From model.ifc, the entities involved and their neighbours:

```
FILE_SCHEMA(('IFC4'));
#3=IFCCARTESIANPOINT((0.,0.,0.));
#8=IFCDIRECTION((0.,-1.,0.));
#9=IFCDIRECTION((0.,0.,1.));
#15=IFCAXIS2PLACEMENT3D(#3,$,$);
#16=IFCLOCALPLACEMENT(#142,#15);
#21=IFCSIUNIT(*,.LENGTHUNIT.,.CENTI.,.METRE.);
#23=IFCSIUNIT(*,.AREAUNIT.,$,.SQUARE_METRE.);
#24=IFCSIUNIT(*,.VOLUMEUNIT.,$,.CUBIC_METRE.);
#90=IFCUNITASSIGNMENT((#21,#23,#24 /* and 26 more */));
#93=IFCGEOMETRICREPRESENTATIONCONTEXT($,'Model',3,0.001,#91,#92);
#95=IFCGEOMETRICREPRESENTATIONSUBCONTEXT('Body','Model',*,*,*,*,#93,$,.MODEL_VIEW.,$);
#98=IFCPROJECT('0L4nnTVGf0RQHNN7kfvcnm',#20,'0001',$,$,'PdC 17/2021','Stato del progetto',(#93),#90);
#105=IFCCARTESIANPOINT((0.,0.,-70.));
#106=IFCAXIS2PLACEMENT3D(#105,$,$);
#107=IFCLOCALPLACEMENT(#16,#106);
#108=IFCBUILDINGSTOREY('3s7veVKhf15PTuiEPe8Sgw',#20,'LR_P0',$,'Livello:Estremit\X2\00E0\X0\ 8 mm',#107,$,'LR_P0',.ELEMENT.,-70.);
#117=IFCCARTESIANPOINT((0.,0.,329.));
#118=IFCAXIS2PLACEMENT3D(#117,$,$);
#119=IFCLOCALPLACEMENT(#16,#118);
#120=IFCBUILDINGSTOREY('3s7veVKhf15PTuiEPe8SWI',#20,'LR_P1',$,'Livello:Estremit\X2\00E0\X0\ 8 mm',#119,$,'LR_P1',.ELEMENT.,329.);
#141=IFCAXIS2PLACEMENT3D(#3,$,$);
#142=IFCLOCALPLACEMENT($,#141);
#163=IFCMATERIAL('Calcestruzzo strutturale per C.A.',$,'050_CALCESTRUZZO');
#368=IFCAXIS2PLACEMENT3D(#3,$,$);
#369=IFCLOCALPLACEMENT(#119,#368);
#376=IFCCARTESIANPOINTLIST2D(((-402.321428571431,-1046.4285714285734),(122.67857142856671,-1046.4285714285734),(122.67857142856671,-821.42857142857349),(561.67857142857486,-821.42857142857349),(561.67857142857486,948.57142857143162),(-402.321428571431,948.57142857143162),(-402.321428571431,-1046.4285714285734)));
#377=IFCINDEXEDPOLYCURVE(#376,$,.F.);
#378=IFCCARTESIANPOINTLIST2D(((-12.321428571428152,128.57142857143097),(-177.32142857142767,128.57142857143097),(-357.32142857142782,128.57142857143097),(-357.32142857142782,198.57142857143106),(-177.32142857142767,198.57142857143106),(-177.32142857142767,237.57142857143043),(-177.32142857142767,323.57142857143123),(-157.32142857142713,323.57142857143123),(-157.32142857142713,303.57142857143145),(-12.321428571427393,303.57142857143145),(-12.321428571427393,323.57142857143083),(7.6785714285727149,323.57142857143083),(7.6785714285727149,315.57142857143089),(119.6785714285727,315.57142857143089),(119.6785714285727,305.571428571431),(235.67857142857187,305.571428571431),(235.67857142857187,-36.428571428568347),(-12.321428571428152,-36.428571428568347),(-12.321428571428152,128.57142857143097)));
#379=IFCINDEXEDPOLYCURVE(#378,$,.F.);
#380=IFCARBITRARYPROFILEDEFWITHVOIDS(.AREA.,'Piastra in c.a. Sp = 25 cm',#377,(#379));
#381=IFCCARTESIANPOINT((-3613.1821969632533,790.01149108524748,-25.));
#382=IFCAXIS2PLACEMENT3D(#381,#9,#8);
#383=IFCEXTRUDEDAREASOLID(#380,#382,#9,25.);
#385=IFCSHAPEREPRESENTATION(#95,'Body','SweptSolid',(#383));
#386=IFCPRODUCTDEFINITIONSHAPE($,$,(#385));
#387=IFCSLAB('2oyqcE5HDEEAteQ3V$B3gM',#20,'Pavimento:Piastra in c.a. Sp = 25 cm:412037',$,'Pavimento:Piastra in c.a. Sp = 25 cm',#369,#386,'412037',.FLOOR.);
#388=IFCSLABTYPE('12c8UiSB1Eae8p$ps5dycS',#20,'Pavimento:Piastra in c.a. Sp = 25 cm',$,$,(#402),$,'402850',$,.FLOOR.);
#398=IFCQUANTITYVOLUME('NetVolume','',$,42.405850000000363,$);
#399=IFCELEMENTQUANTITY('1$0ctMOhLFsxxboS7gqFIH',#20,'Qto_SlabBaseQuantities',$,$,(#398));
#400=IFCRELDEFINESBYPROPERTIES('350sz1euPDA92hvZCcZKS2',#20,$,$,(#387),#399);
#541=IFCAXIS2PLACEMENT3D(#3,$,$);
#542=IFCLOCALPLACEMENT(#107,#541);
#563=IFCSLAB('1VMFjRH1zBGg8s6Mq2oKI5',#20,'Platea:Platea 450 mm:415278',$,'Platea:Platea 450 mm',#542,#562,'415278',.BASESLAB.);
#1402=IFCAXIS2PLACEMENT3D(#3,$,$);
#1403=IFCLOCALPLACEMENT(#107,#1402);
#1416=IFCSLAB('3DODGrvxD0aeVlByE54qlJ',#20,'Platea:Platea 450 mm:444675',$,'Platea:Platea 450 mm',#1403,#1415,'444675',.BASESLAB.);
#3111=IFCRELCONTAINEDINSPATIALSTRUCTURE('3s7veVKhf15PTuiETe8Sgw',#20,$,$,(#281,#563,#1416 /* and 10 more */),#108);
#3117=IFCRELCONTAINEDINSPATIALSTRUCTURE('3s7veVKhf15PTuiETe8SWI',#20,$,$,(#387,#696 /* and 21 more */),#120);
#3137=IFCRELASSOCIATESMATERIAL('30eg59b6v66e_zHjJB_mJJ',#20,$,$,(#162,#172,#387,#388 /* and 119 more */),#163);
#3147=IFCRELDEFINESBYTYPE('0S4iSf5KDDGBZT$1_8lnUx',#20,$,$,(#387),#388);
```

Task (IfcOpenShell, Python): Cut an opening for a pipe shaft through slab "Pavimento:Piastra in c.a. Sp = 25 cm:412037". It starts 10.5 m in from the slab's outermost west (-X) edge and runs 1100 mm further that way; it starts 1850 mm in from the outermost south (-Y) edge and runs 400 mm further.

```python
import numpy as np
import ifcopenshell
import ifcopenshell.api.feature
import ifcopenshell.api.geometry
import ifcopenshell.api.pset
import ifcopenshell.api.root
import ifcopenshell.geom
import ifcopenshell.util.element
import ifcopenshell.util.placement
import ifcopenshell.util.representation
import ifcopenshell.util.shape
import ifcopenshell.util.unit

model = ifcopenshell.open("model.ifc")
unit_scale = ifcopenshell.util.unit.calculate_unit_scale(model)
volume_scale = ifcopenshell.util.unit.calculate_unit_scale(model, "VOLUMEUNIT")
settings = ifcopenshell.geom.settings()


def volume(element):
    """Net volume in cubic metres, openings subtracted."""
    shape = ifcopenshell.geom.create_shape(settings, element)
    return ifcopenshell.util.shape.get_volume(shape.geometry)


slab = model.by_id(387)
before = volume(slab)

# Extent in the slab's own axes, in metres. The edges named are its -X and -Y sides.
slab_shape = ifcopenshell.geom.create_shape(settings, slab)
vertices = ifcopenshell.util.shape.get_vertices(slab_shape.geometry)
x_min, y_min, bottom = vertices.min(axis=0)
top = vertices[:, 2].max()

opening = ifcopenshell.api.root.create_entity(model, ifc_class="IfcOpeningElement", name="Pipe shaft opening", predefined_type="OPENING")
context = ifcopenshell.util.representation.get_context(model, "Model", "Body", "MODEL_VIEW")
width, depth = 1.1, 0.4
outline = [(0.0, 0.0), (width, 0.0), (width, depth), (0.0, depth), (0.0, 0.0)]
# Overshoot both faces by 50 mm so the cut is clean.
shape = ifcopenshell.api.geometry.add_slab_representation(
    model, context=context, depth=top - bottom + 0.1, polyline=outline
)
ifcopenshell.api.geometry.assign_representation(model, product=opening, representation=shape)

matrix = ifcopenshell.util.placement.get_local_placement(slab.ObjectPlacement)
matrix[:, 3] = matrix @ np.append(np.array([x_min + 10.5, y_min + 1.85, bottom - 0.05]) / unit_scale, 1.0)
ifcopenshell.api.geometry.edit_object_placement(model, product=opening, matrix=matrix, is_si=False)
ifcopenshell.api.feature.add_feature(model, feature=opening, element=slab)

after = volume(slab)

# Update the slab's stored quantities.
qto = model.by_id(ifcopenshell.util.element.get_pset(slab, "Qto_SlabBaseQuantities", should_inherit=False)["id"])
ifcopenshell.api.pset.edit_qto(model, qto=qto, properties={"NetVolume": after / volume_scale})

print(f"slab volume {before:.3f} -> {after:.3f} m3")

model.write("model-out.ifc")
```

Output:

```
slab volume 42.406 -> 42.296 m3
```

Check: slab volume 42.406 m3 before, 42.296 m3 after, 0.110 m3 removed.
